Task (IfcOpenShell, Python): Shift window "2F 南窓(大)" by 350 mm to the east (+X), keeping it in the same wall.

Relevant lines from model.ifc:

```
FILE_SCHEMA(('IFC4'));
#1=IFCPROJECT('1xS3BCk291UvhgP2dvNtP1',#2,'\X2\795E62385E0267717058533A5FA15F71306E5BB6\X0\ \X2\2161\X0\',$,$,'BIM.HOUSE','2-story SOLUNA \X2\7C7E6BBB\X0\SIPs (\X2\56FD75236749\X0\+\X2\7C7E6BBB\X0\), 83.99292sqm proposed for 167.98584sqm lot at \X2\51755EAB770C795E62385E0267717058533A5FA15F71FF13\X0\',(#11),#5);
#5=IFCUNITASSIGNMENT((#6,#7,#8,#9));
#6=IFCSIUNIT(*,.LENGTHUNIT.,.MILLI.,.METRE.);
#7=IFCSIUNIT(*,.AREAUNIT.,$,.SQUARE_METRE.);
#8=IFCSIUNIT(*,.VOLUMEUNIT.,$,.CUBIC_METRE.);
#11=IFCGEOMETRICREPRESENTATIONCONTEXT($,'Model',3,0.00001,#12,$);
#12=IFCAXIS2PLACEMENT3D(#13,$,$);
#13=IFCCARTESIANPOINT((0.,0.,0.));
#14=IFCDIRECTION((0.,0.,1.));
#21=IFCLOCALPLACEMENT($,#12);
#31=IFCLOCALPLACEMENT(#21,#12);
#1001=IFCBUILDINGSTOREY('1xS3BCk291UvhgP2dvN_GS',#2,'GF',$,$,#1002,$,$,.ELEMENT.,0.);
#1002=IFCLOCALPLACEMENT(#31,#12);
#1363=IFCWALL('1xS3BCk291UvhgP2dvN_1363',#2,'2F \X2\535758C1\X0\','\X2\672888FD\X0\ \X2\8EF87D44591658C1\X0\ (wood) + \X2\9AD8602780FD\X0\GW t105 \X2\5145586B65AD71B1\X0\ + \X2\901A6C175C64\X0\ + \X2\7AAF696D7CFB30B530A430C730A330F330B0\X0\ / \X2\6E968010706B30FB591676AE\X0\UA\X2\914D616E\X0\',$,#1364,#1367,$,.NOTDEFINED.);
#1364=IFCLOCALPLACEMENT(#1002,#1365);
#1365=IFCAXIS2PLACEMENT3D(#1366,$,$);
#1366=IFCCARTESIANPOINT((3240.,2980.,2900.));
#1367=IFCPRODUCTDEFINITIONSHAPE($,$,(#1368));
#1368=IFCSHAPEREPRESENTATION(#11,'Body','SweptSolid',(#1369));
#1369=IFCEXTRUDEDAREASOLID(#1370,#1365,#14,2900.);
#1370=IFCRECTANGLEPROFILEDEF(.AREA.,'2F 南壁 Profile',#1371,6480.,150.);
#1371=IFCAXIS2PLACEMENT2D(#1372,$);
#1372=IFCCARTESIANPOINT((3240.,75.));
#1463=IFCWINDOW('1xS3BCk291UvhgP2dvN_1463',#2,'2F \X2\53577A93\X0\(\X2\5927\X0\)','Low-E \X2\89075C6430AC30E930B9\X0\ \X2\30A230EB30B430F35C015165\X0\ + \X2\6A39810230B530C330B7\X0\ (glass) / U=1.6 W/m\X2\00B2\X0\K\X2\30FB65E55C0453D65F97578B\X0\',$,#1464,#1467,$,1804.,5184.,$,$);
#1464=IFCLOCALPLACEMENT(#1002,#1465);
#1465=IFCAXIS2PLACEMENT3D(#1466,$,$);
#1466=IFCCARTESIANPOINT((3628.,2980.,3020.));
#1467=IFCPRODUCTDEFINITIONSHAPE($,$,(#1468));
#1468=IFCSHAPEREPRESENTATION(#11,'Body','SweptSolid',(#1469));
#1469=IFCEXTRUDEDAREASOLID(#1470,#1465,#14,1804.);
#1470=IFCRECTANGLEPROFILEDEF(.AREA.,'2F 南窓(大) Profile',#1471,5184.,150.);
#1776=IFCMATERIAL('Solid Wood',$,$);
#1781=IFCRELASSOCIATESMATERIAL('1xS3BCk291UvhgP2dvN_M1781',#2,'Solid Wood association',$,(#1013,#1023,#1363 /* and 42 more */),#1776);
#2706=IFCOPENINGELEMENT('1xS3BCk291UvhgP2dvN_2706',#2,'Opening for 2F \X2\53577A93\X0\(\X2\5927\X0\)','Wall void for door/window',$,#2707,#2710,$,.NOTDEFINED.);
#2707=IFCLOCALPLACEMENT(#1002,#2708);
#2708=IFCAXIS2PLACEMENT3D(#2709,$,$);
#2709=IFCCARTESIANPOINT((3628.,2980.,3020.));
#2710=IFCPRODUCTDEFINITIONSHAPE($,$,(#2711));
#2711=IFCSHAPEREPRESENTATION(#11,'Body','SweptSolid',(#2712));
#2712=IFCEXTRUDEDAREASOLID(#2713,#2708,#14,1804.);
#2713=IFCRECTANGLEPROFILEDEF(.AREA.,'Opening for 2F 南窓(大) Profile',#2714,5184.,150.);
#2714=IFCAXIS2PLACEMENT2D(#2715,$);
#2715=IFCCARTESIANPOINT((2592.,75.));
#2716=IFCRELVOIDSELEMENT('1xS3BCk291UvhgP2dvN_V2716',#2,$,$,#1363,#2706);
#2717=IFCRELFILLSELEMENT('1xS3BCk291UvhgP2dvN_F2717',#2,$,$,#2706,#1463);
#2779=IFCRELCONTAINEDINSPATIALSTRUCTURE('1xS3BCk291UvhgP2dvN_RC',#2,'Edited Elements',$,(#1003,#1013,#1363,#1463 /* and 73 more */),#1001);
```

```python
import ifcopenshell
import ifcopenshell.api.geometry
import ifcopenshell.util.placement
import ifcopenshell.util.unit

model = ifcopenshell.open("model.ifc")
unit_scale = ifcopenshell.util.unit.calculate_unit_scale(model)

window = model.by_guid("1xS3BCk291UvhgP2dvN_1463")
opening = window.FillsVoids[0].RelatingOpeningElement
wall = opening.VoidsElements[0].RelatingBuildingElement

wall_matrix = ifcopenshell.util.placement.get_local_placement(wall.ObjectPlacement)
shift = wall_matrix[:3, 0] * 0.35 / unit_scale
before = ifcopenshell.util.placement.get_local_placement(window.ObjectPlacement)[:3, 3].copy()

# The window is not placed relative to its opening, so move both.
for product in (opening, window):
    matrix = ifcopenshell.util.placement.get_local_placement(product.ObjectPlacement)
    matrix[:3, 3] += shift
    ifcopenshell.api.geometry.edit_object_placement(model, product=product, matrix=matrix, is_si=False)

after = ifcopenshell.util.placement.get_local_placement(window.ObjectPlacement)[:3, 3]
print("window moved by", (after - before).round(3) + 0.0)

model.write("model_v2.ifc")
```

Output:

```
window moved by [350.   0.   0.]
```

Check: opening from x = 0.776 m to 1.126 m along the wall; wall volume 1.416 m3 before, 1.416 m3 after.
